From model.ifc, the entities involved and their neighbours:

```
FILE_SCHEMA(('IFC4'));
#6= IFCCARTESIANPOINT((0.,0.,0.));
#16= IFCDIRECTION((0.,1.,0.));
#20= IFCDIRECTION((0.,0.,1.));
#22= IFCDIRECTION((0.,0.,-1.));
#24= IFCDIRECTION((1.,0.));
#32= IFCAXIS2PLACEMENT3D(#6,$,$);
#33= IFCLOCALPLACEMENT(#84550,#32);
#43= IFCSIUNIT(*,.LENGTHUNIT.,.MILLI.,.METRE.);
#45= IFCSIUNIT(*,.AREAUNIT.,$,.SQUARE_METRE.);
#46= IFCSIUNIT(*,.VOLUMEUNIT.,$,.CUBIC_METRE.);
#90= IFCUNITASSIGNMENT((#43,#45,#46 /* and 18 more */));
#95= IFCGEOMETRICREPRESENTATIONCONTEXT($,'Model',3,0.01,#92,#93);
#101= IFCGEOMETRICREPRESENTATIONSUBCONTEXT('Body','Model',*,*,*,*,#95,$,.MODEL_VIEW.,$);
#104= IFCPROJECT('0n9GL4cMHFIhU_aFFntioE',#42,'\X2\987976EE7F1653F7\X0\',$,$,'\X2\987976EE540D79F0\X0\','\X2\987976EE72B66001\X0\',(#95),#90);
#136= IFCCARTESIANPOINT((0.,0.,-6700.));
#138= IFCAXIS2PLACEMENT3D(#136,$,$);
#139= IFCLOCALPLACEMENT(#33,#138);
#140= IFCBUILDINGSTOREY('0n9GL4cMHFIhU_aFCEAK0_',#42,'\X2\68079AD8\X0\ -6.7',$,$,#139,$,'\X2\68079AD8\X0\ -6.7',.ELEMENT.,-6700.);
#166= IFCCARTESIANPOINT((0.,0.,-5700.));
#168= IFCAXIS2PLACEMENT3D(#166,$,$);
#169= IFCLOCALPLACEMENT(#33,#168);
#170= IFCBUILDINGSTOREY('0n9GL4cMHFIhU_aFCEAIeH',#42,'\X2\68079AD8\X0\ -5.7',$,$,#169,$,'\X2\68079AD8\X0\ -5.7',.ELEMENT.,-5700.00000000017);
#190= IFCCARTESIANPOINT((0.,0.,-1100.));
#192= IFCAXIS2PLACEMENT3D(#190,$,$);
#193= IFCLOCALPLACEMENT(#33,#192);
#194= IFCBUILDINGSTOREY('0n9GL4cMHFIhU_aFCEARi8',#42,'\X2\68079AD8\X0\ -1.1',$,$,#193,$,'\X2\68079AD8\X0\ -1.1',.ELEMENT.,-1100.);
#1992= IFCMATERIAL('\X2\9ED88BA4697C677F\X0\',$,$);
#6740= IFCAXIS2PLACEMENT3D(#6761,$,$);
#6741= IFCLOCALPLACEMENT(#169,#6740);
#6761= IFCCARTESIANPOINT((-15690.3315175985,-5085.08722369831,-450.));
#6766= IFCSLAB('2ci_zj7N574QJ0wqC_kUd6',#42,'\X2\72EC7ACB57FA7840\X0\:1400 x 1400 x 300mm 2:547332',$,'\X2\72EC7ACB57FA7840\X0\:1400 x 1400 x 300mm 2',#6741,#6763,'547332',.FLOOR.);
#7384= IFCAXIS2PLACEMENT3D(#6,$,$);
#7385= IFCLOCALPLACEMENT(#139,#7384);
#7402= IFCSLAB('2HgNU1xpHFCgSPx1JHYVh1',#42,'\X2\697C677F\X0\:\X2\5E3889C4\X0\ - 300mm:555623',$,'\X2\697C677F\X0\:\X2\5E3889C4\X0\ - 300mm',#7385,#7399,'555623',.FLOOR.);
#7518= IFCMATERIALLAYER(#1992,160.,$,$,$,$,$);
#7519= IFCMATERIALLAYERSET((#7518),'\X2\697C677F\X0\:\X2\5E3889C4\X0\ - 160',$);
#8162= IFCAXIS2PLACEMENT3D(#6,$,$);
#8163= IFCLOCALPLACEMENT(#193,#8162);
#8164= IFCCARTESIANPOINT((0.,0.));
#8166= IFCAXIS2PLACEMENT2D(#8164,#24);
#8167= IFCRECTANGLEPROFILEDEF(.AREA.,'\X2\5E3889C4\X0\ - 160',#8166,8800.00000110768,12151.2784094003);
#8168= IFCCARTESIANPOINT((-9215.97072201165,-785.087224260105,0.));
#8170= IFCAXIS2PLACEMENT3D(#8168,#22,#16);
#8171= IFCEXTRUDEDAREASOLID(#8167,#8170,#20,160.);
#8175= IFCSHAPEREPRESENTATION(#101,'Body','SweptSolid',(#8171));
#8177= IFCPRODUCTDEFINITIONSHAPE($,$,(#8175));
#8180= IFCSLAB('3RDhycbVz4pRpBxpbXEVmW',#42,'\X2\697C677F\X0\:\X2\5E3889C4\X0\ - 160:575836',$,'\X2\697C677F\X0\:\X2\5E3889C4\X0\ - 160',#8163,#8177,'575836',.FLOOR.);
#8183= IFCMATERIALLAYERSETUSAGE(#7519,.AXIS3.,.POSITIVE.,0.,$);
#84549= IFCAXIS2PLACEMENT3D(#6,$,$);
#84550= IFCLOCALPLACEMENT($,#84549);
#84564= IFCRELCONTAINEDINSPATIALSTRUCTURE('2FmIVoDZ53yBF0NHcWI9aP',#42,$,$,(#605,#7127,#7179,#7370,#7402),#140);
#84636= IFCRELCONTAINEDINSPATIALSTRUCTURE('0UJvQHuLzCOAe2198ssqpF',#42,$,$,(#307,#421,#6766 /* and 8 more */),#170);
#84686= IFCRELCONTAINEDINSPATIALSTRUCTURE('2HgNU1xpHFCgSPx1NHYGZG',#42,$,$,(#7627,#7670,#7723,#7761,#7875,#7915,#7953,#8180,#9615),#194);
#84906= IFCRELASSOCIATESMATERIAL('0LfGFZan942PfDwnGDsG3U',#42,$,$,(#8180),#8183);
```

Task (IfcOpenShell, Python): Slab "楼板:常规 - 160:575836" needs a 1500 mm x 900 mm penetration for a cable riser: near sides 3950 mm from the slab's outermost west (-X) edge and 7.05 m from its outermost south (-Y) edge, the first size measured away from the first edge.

```python
import numpy as np
import ifcopenshell
import ifcopenshell.api.feature
import ifcopenshell.api.geometry
import ifcopenshell.api.root
import ifcopenshell.geom
import ifcopenshell.util.placement
import ifcopenshell.util.representation
import ifcopenshell.util.shape
import ifcopenshell.util.unit

model = ifcopenshell.open("model.ifc")
unit_scale = ifcopenshell.util.unit.calculate_unit_scale(model)
settings = ifcopenshell.geom.settings()


def volume(element):
    """Net volume in cubic metres, openings subtracted."""
    shape = ifcopenshell.geom.create_shape(settings, element)
    return ifcopenshell.util.shape.get_volume(shape.geometry)


slab = model.by_id(8180)
before = volume(slab)

# Extent in the slab's own axes, in metres. The edges named are its -X and -Y sides.
slab_shape = ifcopenshell.geom.create_shape(settings, slab)
vertices = ifcopenshell.util.shape.get_vertices(slab_shape.geometry)
x_min, y_min, bottom = vertices.min(axis=0)
top = vertices[:, 2].max()

opening = ifcopenshell.api.root.create_entity(model, ifc_class="IfcOpeningElement", name="Cable riser opening", predefined_type="OPENING")
context = ifcopenshell.util.representation.get_context(model, "Model", "Body", "MODEL_VIEW")
width, depth = 1.5, 0.9
outline = [(0.0, 0.0), (width, 0.0), (width, depth), (0.0, depth), (0.0, 0.0)]
# Overshoot both faces by 50 mm so the cut is clean.
shape = ifcopenshell.api.geometry.add_slab_representation(
    model, context=context, depth=top - bottom + 0.1, polyline=outline
)
ifcopenshell.api.geometry.assign_representation(model, product=opening, representation=shape)

matrix = ifcopenshell.util.placement.get_local_placement(slab.ObjectPlacement)
matrix[:, 3] = matrix @ np.append(np.array([x_min + 3.95, y_min + 7.05, bottom - 0.05]) / unit_scale, 1.0)
ifcopenshell.api.geometry.edit_object_placement(model, product=opening, matrix=matrix, is_si=False)
ifcopenshell.api.feature.add_feature(model, feature=opening, element=slab)

after = volume(slab)

print(f"slab volume {before:.3f} -> {after:.3f} m3")

model.write("model-out.ifc")
```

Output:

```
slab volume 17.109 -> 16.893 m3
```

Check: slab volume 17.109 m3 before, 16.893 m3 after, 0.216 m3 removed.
